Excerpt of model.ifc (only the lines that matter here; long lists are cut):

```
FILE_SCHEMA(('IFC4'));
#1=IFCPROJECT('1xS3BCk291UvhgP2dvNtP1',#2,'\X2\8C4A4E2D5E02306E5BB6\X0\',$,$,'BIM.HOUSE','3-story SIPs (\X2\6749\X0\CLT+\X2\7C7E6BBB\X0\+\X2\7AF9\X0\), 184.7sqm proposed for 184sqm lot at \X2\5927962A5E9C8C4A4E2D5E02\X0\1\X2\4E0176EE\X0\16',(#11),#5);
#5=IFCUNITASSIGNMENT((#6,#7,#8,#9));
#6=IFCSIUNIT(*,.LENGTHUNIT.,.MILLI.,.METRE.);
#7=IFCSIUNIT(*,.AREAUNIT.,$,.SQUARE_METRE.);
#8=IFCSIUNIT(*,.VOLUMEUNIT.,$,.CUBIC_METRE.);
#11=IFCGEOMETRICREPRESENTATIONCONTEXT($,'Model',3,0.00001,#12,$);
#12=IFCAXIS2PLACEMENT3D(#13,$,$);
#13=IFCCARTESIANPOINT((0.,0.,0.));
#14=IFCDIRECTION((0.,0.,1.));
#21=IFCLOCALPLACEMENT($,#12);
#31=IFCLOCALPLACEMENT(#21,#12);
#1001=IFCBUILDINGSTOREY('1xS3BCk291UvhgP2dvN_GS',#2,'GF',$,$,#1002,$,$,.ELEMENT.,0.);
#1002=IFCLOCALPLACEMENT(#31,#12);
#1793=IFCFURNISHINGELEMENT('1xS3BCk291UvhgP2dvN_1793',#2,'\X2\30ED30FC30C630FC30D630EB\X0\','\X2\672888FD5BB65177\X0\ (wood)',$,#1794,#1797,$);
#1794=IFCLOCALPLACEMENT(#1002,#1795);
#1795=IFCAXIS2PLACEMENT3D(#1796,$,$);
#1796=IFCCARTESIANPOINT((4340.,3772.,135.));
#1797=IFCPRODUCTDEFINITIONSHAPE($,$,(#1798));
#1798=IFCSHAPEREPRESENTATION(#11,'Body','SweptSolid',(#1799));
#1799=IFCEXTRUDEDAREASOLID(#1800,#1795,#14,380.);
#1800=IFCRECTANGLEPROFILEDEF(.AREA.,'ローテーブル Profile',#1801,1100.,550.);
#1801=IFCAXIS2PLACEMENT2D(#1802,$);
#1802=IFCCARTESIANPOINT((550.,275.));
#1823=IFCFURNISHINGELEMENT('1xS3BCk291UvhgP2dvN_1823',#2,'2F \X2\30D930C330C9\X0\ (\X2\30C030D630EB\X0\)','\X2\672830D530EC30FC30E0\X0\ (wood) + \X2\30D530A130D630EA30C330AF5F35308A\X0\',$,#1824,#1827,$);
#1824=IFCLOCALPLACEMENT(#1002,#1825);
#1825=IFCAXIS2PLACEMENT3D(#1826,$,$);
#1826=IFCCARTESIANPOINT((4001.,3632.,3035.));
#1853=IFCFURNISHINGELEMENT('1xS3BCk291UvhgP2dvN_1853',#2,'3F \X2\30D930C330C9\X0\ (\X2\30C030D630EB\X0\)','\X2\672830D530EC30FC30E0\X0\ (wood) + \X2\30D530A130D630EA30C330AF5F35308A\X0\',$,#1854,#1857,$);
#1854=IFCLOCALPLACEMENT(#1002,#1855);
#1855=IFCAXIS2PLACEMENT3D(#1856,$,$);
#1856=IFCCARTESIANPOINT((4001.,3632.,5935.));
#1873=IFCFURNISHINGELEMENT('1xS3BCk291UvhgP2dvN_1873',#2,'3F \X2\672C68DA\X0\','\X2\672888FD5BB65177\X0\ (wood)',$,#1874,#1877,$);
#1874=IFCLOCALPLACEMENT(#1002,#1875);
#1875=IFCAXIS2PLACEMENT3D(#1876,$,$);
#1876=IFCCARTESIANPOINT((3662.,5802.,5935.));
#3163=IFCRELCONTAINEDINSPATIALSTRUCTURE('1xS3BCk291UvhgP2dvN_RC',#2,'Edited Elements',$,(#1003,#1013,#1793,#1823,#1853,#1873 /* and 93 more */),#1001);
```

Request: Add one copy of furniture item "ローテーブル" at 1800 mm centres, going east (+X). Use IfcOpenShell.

```python
import numpy as np
import ifcopenshell
import ifcopenshell.api.geometry
import ifcopenshell.api.root
import ifcopenshell.util.element
import ifcopenshell.util.placement

model = ifcopenshell.open("model.ifc")


def reuse_history(source, copy):
    """copy_class also copies each property set's owner history, people and application; keep the originals."""
    for rel in copy.IsDefinedBy:
        if rel.is_a("IfcRelDefinesByProperties") and (history := rel.RelatingPropertyDefinition.OwnerHistory):
            rel.RelatingPropertyDefinition.OwnerHistory = source.OwnerHistory
            ifcopenshell.util.element.remove_deep2(model, history)


source = model.by_id(1793)
base = ifcopenshell.util.placement.get_local_placement(source.ObjectPlacement)
step = np.array([1.0, 0.0, 0.0]) * 1800.0

for i in range(1, 2):
    copy = ifcopenshell.api.root.copy_class(model, product=source)
    copy.Representation = ifcopenshell.util.element.copy_deep(
        model, source.Representation, exclude=["IfcGeometricRepresentationContext", "IfcRepresentationMap"]
    )
    reuse_history(source, copy)
    matrix = base.copy()
    matrix[:3, 3] += i * step
    print("added at", matrix[:3, 3].round(3) + 0.0)
    ifcopenshell.api.geometry.edit_object_placement(model, product=copy, matrix=matrix, is_si=False)

model.write("model-out.ifc")
```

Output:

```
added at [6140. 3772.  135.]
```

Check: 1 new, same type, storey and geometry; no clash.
